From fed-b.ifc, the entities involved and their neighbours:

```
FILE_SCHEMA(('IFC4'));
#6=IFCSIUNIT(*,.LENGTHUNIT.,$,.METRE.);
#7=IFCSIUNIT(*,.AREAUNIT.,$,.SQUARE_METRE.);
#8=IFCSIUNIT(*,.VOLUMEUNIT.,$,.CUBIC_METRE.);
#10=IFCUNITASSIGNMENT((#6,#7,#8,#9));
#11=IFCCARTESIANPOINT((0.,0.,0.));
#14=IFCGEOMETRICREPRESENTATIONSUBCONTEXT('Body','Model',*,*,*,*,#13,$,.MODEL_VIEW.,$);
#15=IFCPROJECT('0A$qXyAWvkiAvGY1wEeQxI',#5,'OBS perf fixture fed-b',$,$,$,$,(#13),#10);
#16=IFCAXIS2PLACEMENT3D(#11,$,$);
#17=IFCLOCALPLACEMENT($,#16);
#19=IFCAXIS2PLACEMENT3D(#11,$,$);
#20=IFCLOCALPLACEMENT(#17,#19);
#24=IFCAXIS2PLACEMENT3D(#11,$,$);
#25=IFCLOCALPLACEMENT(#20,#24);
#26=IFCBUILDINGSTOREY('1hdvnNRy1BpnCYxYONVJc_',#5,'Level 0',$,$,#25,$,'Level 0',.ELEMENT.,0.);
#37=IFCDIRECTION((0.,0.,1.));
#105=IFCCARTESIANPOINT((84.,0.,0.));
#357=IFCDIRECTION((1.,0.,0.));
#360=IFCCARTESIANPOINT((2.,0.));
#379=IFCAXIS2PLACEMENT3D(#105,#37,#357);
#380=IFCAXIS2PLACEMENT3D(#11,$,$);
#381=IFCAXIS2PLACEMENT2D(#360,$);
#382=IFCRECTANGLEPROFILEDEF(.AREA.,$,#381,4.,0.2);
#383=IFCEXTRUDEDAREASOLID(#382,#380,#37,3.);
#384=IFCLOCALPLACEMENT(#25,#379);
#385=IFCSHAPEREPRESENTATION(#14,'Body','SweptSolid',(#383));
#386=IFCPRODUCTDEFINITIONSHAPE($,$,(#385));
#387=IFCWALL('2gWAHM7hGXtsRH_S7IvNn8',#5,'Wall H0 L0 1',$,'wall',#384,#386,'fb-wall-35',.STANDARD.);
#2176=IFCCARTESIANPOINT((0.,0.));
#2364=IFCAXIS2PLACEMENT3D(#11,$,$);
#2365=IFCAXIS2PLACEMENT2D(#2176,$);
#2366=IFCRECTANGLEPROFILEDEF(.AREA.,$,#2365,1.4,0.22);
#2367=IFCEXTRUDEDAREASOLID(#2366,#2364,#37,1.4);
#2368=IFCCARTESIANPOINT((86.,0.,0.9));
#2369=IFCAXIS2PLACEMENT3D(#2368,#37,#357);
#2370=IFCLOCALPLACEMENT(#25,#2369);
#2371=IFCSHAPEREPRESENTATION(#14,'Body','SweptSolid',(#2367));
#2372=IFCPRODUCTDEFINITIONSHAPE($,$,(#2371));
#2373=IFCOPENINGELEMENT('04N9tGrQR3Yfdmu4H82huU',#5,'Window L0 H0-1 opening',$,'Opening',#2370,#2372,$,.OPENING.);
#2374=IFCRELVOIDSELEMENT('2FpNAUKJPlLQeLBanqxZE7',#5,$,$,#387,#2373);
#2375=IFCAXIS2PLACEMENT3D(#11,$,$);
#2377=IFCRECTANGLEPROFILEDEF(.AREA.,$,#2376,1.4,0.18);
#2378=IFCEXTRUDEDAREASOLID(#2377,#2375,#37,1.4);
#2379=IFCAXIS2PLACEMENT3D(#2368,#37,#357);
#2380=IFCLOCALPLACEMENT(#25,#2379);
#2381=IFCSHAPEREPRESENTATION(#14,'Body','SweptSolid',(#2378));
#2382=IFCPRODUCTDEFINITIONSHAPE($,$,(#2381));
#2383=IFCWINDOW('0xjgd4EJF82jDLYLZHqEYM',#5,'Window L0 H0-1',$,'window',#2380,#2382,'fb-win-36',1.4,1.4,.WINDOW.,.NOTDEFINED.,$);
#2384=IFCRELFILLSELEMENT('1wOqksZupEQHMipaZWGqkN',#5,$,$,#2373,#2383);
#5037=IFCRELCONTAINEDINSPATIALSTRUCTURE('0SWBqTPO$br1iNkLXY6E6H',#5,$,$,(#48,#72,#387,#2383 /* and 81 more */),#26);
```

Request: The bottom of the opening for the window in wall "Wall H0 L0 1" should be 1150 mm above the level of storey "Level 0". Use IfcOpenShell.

```python
import numpy as np
import ifcopenshell
import ifcopenshell.api.geometry
import ifcopenshell.geom
import ifcopenshell.util.element
import ifcopenshell.util.placement
import ifcopenshell.util.shape
import ifcopenshell.util.unit

model = ifcopenshell.open("fed-b.ifc")
unit_scale = ifcopenshell.util.unit.calculate_unit_scale(model)

window = model.by_guid("0xjgd4EJF82jDLYLZHqEYM")
opening = window.FillsVoids[0].RelatingOpeningElement
storey = ifcopenshell.util.element.get_container(window, ifc_class="IfcBuildingStorey")
level = ifcopenshell.util.placement.get_local_placement(storey.ObjectPlacement)[2, 3]

# The opening's origin need not be at the sill, so measure its lowest point.
shape = ifcopenshell.geom.create_shape(ifcopenshell.geom.settings(), opening)
bottom = ifcopenshell.util.shape.get_shape_bottom_elevation(shape, shape.geometry) / unit_scale
dz = level + 1.15 - bottom

shift = np.array([0.0, 0.0, dz])
# The window is not placed relative to its opening, so move both.
for product in (opening, window):
    matrix = ifcopenshell.util.placement.get_local_placement(product.ObjectPlacement)
    matrix[:3, 3] += shift
    ifcopenshell.api.geometry.edit_object_placement(model, product=product, matrix=matrix, is_si=False)

print(f"moved by {dz * unit_scale:+.3f} m")

model.write("fed-b_v2.ifc")
```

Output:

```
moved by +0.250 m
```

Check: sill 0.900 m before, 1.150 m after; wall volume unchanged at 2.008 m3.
